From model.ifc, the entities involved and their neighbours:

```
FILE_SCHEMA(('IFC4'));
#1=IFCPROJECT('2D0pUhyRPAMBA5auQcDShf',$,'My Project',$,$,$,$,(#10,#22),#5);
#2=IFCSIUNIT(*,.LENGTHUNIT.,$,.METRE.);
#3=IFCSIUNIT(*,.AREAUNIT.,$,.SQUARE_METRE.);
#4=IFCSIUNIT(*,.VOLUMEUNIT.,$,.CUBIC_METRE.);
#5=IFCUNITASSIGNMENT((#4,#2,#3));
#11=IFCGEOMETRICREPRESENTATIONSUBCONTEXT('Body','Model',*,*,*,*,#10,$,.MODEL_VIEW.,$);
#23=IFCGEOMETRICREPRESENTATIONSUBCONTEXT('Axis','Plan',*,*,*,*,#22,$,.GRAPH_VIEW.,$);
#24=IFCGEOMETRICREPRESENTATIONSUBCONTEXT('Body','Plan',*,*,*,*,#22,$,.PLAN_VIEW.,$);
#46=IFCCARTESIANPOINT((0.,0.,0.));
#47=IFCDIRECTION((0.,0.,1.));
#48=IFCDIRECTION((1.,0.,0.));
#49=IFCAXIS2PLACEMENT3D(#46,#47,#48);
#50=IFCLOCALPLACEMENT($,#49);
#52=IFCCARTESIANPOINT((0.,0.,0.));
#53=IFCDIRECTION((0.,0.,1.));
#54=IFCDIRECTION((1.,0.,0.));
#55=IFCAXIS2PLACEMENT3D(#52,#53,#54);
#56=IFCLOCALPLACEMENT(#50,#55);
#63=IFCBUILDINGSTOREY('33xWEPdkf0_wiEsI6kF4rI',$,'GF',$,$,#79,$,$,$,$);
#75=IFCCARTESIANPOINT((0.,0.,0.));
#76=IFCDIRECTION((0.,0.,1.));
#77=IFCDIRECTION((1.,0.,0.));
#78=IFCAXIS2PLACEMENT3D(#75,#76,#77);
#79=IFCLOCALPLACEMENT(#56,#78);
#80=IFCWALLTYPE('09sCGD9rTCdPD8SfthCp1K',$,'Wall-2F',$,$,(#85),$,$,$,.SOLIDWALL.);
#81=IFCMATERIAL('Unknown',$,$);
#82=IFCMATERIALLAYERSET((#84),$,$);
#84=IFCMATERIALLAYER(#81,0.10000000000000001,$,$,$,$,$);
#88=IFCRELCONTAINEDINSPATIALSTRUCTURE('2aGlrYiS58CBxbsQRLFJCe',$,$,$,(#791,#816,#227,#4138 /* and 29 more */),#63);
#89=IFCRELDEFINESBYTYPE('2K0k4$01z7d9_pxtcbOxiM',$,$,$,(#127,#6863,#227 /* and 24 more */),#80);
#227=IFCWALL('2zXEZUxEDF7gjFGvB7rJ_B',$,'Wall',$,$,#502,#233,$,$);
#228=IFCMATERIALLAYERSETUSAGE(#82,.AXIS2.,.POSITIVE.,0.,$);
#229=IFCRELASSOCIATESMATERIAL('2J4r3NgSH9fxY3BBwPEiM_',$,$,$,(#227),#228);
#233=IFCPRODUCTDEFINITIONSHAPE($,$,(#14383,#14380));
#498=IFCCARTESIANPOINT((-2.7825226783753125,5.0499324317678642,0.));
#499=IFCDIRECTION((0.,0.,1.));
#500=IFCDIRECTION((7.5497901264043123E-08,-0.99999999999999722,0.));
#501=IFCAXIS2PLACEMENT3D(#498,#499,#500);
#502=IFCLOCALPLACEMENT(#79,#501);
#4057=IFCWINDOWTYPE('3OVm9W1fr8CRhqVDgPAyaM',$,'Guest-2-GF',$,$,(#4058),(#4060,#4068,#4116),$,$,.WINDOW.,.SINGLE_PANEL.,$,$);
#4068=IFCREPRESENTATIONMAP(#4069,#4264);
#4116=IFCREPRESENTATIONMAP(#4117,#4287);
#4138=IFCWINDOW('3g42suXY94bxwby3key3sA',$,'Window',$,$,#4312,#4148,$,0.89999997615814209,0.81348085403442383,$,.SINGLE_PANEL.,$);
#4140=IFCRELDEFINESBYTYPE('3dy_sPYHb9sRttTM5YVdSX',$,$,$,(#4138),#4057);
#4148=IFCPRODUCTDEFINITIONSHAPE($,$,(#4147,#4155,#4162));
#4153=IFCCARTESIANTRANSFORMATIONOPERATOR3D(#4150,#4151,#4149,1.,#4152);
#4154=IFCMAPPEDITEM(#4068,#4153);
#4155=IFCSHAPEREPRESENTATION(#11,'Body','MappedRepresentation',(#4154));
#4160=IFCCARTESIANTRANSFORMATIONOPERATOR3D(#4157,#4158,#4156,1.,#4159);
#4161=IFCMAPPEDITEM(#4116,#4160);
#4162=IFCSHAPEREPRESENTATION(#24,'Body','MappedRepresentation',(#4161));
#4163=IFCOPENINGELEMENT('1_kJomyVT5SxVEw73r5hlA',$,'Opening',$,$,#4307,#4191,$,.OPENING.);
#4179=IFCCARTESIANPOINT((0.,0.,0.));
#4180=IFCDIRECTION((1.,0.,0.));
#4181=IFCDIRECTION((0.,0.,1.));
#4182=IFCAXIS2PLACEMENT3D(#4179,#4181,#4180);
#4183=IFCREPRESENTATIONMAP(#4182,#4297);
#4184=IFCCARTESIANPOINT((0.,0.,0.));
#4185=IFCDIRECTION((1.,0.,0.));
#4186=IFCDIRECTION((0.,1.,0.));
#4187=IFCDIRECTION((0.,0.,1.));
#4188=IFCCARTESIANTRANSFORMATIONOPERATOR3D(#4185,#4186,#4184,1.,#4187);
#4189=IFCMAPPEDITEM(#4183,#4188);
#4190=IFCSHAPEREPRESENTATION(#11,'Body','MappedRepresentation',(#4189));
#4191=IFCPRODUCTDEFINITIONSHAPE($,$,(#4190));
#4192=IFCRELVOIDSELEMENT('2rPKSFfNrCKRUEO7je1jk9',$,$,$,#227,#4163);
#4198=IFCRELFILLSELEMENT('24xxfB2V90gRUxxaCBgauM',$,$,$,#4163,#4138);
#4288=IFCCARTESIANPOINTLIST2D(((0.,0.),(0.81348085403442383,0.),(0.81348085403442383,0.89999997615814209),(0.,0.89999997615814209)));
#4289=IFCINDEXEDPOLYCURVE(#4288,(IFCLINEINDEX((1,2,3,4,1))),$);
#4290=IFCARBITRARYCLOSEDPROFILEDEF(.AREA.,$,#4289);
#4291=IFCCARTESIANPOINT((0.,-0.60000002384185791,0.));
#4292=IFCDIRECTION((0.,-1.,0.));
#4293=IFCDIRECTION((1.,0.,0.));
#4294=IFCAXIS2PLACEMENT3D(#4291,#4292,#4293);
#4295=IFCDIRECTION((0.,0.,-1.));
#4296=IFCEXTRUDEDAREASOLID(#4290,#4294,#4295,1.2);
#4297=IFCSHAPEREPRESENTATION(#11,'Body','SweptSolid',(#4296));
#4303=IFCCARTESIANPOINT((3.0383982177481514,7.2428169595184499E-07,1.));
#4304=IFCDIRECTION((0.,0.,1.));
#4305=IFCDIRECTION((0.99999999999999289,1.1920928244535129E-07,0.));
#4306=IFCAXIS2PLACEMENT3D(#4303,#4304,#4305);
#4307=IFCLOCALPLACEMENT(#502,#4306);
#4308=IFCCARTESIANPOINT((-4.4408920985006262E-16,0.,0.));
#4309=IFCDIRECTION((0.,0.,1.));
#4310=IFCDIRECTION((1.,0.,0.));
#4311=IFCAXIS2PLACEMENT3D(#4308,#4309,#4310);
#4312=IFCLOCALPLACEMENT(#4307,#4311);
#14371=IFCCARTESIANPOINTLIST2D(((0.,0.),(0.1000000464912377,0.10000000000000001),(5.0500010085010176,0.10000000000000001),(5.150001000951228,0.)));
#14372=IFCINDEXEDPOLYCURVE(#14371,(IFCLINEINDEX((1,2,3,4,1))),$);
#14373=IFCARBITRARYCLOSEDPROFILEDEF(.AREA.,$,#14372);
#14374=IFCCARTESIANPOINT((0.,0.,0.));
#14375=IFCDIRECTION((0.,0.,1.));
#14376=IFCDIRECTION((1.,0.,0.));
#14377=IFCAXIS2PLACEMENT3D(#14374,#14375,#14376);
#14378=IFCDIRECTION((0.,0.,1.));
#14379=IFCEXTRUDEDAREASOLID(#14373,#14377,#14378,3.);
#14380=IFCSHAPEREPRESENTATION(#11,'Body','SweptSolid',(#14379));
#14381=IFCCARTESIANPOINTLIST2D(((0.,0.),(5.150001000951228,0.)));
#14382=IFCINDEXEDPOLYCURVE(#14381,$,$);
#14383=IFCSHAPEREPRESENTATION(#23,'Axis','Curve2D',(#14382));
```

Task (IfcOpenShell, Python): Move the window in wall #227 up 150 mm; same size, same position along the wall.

```python
import numpy as np
import ifcopenshell
import ifcopenshell.api.geometry
import ifcopenshell.util.placement
import ifcopenshell.util.unit

model = ifcopenshell.open("model.ifc")
unit_scale = ifcopenshell.util.unit.calculate_unit_scale(model)

window = model.by_id(4138)
opening = window.FillsVoids[0].RelatingOpeningElement
dz = 0.15

shift = np.array([0.0, 0.0, dz])
# The window is placed relative to its opening, so it follows when the opening moves.
matrix = ifcopenshell.util.placement.get_local_placement(opening.ObjectPlacement)
matrix[:3, 3] += shift
ifcopenshell.api.geometry.edit_object_placement(
    model, product=opening, matrix=matrix, is_si=False, should_transform_children=True
)

print(f"moved by {dz * unit_scale:+.3f} m")

model.write("model_rev.ifc")
```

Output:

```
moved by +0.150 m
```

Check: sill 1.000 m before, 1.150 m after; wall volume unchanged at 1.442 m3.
